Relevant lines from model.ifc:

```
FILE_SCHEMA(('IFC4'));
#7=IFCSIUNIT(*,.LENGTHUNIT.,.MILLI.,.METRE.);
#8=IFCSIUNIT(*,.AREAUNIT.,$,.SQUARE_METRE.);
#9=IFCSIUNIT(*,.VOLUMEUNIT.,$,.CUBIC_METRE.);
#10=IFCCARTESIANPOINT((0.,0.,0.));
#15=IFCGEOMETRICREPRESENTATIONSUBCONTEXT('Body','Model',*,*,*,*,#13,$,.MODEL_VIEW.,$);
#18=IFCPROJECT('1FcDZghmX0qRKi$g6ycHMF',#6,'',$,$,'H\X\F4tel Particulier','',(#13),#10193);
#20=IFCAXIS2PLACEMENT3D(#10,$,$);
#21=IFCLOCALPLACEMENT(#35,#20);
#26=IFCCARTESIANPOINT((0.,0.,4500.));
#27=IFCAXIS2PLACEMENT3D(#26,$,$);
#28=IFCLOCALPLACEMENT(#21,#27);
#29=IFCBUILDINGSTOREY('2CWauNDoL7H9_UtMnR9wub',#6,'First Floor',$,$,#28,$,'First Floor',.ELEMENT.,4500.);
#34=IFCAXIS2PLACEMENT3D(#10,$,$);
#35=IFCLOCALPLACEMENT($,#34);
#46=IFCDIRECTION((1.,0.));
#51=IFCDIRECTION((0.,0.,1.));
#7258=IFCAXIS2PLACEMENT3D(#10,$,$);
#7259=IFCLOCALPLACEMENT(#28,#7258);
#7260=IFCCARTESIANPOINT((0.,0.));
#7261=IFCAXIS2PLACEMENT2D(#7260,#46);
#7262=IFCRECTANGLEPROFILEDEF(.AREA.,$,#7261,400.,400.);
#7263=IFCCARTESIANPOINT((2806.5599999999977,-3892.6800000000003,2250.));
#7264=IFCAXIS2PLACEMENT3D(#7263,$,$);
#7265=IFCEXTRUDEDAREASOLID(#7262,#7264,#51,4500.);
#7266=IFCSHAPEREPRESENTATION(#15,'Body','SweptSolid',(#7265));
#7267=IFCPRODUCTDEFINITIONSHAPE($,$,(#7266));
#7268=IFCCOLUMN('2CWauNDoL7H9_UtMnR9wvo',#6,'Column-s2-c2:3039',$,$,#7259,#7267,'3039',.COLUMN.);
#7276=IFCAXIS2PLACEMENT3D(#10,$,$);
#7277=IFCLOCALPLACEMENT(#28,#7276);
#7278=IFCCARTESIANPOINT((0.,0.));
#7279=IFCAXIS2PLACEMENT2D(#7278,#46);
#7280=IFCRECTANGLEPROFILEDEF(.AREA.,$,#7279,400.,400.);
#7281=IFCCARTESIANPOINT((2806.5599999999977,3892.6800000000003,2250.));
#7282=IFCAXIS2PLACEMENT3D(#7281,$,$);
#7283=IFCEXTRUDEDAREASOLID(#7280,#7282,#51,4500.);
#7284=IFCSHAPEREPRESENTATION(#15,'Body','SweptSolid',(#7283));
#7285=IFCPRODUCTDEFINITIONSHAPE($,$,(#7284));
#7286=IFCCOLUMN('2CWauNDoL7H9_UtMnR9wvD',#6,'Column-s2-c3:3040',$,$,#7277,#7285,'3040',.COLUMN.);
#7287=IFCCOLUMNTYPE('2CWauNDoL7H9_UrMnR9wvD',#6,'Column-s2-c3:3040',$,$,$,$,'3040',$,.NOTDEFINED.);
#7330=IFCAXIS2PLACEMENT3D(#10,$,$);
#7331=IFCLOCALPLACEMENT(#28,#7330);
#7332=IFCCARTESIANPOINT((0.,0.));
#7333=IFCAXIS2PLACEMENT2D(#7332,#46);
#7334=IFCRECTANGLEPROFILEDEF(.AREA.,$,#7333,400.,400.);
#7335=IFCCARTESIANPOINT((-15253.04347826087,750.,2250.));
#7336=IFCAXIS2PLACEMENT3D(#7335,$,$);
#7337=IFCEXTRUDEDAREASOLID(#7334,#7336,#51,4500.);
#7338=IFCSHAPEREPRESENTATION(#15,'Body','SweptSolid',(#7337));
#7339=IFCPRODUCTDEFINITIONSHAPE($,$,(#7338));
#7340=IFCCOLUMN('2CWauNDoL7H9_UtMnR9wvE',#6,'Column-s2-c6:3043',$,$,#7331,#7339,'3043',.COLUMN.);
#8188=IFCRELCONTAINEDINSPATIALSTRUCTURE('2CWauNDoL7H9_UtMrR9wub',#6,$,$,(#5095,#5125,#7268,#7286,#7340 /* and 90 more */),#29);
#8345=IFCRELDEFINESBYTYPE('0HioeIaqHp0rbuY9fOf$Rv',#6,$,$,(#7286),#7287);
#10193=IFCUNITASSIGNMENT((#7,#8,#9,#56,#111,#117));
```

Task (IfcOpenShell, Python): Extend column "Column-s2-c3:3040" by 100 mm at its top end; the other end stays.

```python
import ifcopenshell
import ifcopenshell.util.representation
import ifcopenshell.util.unit

model = ifcopenshell.open("model.ifc")
unit_scale = ifcopenshell.util.unit.calculate_unit_scale(model)

member = model.by_guid("2CWauNDoL7H9_UtMnR9wvD")
change = 0.1 / unit_scale

# The extrusion runs towards the end named, so only its depth changes.
body = ifcopenshell.util.representation.get_representation(member, "Model", "Body")
solid = body.Items[0]
old_length = solid.Depth
solid.Depth += change

print(f"length {old_length:g} -> {solid.Depth:g}")

model.write("model_updated.ifc")
```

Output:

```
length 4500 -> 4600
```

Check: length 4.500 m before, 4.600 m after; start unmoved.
